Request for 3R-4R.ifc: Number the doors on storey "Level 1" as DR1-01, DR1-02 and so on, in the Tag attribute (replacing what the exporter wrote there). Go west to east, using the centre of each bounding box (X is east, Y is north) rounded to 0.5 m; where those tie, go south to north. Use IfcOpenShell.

First a look at what the model holds.

```python
import ifcopenshell
import ifcopenshell.util.element
import ifcopenshell.util.placement

model = ifcopenshell.open("3R-4R.ifc")
print(model.schema)
storey = next(s for s in model.by_type("IfcBuildingStorey") if s.Name == "Level 1")
doors = [e for e in ifcopenshell.util.element.get_decomposition(storey) if e.is_a("IfcDoor")]
for e in sorted(doors, key=lambda e: e.id()):
    origin = ifcopenshell.util.placement.get_local_placement(e.ObjectPlacement)[:3, 3]
    print(e.id(), e.Tag, e.Name, origin.round(2) + 0.0, sep=" | ")
```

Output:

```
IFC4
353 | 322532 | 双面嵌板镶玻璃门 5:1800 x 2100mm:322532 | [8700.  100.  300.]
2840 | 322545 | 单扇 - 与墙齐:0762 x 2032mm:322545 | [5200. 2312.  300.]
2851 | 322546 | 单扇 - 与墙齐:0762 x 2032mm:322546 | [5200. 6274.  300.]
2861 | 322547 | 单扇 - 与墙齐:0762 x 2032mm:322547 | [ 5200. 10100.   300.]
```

```python
import ifcopenshell
import ifcopenshell.geom
import ifcopenshell.util.element
import ifcopenshell.util.shape

model = ifcopenshell.open("3R-4R.ifc")
settings = ifcopenshell.geom.settings()
settings.set("use-world-coords", True)


def centre(element):
    shape = ifcopenshell.geom.create_shape(settings, element)
    return ifcopenshell.util.shape.get_bbox_centroid(shape.geometry)


storey = next(s for s in model.by_type("IfcBuildingStorey") if s.Name == "Level 1")
doors = [e for e in ifcopenshell.util.element.get_decomposition(storey) if e.is_a("IfcDoor")]

# Insertion points can sit at a corner or the storey origin, so sort by the geometry (in metres).
centres = {e: centre(e) for e in doors}
doors.sort(key=lambda e: (round(centres[e][0] / 0.5), centres[e][1]))

for i, e in enumerate(doors, start=1):
    number = f"DR1-{i:02d}"
    e.Tag = number
    print(e.id(), number)

model.write("3R-4R_rev.ifc")
```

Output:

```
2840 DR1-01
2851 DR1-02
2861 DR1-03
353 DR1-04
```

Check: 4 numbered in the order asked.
